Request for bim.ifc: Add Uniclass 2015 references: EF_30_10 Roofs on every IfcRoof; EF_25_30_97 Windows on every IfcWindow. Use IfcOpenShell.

First a look at what the model holds.

```python
import ifcopenshell

model = ifcopenshell.open("bim.ifc")
print(model.schema)
print("classifications:", [c.Name for c in model.by_type("IfcClassification")])
for ifc_class in ("IfcDoor", "IfcRoof", "IfcStair", "IfcWall", "IfcWindow"):
    print(ifc_class, len(model.by_type(ifc_class)))
```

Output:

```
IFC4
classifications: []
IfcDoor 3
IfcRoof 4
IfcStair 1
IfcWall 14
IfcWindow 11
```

```python
import ifcopenshell
import ifcopenshell.api.classification

model = ifcopenshell.open("bim.ifc")

system = ifcopenshell.api.classification.add_classification(model, classification="Uniclass 2015")

codes = {
    "IfcRoof": ("EF_30_10", "Roofs"),
    "IfcWindow": ("EF_25_30_97", "Windows"),
}
for ifc_class, (code, name) in codes.items():
    products = model.by_type(ifc_class)
    ifcopenshell.api.classification.add_reference(
        model, products=products, classification=system, identification=code, name=name
    )
    print(code, len(products))

model.write("bim_edited.ifc")
```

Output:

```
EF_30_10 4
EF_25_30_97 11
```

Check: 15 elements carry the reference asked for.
